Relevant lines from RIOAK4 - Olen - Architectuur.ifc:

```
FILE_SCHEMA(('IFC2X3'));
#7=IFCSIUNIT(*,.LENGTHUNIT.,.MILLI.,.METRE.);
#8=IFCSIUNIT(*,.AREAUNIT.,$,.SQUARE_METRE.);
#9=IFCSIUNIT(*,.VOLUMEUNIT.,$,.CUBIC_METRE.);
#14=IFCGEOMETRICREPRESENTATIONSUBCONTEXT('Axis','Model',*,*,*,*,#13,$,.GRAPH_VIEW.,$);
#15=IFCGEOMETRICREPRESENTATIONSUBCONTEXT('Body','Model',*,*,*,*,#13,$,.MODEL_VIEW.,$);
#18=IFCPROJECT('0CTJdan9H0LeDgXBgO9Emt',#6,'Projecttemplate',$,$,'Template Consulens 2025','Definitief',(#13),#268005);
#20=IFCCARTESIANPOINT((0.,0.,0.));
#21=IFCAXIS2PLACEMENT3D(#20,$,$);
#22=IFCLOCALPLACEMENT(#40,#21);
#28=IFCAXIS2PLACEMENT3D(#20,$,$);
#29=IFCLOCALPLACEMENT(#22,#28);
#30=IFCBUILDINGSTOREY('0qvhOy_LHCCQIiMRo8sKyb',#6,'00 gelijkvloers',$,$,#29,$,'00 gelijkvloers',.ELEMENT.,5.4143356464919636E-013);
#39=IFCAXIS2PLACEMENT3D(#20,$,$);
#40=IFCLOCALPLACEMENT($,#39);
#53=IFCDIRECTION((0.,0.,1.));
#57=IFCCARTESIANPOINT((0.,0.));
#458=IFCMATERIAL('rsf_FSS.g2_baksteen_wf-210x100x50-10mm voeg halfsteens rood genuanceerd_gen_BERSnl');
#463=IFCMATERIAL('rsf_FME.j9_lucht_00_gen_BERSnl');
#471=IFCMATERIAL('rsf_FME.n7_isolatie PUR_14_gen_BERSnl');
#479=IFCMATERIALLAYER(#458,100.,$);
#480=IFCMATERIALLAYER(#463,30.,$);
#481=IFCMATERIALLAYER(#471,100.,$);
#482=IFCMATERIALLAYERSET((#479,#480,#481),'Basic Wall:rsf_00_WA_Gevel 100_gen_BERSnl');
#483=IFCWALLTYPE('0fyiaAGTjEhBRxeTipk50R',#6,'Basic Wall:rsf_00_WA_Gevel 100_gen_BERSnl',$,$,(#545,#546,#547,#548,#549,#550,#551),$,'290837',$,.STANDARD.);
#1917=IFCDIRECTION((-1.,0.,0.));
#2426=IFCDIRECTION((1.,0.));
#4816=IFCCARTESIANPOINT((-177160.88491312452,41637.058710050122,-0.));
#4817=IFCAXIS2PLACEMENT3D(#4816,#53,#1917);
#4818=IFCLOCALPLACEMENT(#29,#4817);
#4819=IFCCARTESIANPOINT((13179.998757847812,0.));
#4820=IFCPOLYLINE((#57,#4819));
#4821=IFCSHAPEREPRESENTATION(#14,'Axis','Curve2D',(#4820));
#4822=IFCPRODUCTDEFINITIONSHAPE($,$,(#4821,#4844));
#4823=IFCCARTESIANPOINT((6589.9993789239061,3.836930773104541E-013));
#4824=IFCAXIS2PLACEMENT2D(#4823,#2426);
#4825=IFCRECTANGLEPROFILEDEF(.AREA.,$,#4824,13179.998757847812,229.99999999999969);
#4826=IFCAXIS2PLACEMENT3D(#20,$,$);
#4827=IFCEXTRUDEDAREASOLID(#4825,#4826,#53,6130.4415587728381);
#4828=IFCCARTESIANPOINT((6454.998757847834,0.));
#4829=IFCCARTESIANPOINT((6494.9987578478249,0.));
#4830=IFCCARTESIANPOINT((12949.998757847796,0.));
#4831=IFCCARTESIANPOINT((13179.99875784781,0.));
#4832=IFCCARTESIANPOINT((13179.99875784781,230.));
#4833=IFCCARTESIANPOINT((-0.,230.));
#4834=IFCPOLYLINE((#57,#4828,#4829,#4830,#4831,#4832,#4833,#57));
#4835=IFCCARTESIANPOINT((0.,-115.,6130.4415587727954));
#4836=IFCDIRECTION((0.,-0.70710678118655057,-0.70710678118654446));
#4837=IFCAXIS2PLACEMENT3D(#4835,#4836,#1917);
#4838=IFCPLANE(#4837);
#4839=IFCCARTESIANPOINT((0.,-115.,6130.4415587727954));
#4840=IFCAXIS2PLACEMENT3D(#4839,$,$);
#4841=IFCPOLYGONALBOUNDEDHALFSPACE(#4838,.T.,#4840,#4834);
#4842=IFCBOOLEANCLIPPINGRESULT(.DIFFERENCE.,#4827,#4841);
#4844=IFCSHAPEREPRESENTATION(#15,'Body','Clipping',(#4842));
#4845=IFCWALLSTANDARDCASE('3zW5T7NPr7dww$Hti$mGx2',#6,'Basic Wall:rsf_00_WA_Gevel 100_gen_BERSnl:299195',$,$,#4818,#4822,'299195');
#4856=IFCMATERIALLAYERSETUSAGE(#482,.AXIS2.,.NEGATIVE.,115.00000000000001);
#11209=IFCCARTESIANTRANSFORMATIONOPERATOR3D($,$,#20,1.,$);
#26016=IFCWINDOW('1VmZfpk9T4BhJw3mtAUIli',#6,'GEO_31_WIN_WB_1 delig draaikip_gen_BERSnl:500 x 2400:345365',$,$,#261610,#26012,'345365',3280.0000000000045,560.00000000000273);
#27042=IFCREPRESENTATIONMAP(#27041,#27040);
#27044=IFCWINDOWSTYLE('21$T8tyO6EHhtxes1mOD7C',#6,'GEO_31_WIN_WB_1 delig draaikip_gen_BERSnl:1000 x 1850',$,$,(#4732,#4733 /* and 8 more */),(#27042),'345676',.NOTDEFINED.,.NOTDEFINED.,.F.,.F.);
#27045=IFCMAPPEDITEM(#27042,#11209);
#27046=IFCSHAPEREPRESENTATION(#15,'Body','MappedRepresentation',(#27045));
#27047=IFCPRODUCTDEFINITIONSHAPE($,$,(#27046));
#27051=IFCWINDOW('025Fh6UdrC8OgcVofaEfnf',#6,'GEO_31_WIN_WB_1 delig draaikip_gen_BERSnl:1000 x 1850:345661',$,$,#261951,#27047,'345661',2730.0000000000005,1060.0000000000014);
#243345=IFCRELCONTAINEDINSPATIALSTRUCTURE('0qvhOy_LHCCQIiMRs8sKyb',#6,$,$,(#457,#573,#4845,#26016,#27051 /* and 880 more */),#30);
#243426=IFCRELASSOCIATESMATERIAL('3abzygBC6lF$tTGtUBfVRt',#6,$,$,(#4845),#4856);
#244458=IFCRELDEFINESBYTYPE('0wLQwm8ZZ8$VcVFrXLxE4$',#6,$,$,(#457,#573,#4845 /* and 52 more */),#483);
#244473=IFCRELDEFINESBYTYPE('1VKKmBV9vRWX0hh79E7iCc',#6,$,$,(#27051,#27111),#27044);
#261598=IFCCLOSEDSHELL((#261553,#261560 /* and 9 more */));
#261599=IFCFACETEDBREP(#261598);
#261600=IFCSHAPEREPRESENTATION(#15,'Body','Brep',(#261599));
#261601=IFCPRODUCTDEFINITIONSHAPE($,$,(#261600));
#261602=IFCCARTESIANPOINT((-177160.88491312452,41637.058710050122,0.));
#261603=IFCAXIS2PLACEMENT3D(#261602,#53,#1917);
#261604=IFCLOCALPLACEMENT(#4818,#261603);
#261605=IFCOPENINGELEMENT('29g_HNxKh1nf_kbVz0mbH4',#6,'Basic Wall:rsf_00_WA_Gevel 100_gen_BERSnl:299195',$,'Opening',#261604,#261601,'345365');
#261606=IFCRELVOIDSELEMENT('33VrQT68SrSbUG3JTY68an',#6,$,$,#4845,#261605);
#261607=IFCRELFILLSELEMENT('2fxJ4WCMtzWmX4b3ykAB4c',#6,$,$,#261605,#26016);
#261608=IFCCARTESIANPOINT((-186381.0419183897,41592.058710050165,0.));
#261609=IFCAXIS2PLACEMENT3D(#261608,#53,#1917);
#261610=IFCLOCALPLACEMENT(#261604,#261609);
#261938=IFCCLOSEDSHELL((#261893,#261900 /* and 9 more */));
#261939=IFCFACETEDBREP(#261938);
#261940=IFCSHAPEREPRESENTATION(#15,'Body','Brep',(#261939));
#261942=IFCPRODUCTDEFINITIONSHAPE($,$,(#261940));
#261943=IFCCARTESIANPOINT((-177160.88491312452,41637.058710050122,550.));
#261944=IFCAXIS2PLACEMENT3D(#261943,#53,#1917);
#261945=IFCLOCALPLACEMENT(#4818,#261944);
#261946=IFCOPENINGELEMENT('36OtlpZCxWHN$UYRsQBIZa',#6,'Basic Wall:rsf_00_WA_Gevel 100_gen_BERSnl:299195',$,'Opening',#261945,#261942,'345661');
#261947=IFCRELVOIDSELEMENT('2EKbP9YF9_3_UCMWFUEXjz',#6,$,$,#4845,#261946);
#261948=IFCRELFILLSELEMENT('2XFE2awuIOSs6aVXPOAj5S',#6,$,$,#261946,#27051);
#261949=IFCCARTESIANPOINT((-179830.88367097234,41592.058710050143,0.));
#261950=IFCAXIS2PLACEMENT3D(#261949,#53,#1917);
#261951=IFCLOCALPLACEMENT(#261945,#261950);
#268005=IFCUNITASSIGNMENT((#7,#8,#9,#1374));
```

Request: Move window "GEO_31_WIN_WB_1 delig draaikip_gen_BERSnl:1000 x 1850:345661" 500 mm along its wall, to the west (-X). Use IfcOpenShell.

```python
import ifcopenshell
import ifcopenshell.api.geometry
import ifcopenshell.util.placement

model = ifcopenshell.open("RIOAK4 - Olen - Architectuur.ifc")

window = model.by_guid("025Fh6UdrC8OgcVofaEfnf")
opening = window.FillsVoids[0].RelatingOpeningElement
wall = opening.VoidsElements[0].RelatingBuildingElement

wall_matrix = ifcopenshell.util.placement.get_local_placement(wall.ObjectPlacement)
shift = wall_matrix[:3, 0] * 500.0
before = ifcopenshell.util.placement.get_local_placement(window.ObjectPlacement)[:3, 3].copy()

# The window is placed relative to its opening, so it follows when the opening moves.
matrix = ifcopenshell.util.placement.get_local_placement(opening.ObjectPlacement)
matrix[:3, 3] += shift
ifcopenshell.api.geometry.edit_object_placement(
    model, product=opening, matrix=matrix, is_si=False, should_transform_children=True
)

after = ifcopenshell.util.placement.get_local_placement(window.ObjectPlacement)[:3, 3]
print("window moved by", (after - before).round(3) + 0.0)

model.write("RIOAK4 - Olen - Architectuur_rev.ifc")
```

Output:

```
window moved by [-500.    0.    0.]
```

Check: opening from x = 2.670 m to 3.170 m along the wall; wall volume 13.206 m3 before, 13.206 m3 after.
